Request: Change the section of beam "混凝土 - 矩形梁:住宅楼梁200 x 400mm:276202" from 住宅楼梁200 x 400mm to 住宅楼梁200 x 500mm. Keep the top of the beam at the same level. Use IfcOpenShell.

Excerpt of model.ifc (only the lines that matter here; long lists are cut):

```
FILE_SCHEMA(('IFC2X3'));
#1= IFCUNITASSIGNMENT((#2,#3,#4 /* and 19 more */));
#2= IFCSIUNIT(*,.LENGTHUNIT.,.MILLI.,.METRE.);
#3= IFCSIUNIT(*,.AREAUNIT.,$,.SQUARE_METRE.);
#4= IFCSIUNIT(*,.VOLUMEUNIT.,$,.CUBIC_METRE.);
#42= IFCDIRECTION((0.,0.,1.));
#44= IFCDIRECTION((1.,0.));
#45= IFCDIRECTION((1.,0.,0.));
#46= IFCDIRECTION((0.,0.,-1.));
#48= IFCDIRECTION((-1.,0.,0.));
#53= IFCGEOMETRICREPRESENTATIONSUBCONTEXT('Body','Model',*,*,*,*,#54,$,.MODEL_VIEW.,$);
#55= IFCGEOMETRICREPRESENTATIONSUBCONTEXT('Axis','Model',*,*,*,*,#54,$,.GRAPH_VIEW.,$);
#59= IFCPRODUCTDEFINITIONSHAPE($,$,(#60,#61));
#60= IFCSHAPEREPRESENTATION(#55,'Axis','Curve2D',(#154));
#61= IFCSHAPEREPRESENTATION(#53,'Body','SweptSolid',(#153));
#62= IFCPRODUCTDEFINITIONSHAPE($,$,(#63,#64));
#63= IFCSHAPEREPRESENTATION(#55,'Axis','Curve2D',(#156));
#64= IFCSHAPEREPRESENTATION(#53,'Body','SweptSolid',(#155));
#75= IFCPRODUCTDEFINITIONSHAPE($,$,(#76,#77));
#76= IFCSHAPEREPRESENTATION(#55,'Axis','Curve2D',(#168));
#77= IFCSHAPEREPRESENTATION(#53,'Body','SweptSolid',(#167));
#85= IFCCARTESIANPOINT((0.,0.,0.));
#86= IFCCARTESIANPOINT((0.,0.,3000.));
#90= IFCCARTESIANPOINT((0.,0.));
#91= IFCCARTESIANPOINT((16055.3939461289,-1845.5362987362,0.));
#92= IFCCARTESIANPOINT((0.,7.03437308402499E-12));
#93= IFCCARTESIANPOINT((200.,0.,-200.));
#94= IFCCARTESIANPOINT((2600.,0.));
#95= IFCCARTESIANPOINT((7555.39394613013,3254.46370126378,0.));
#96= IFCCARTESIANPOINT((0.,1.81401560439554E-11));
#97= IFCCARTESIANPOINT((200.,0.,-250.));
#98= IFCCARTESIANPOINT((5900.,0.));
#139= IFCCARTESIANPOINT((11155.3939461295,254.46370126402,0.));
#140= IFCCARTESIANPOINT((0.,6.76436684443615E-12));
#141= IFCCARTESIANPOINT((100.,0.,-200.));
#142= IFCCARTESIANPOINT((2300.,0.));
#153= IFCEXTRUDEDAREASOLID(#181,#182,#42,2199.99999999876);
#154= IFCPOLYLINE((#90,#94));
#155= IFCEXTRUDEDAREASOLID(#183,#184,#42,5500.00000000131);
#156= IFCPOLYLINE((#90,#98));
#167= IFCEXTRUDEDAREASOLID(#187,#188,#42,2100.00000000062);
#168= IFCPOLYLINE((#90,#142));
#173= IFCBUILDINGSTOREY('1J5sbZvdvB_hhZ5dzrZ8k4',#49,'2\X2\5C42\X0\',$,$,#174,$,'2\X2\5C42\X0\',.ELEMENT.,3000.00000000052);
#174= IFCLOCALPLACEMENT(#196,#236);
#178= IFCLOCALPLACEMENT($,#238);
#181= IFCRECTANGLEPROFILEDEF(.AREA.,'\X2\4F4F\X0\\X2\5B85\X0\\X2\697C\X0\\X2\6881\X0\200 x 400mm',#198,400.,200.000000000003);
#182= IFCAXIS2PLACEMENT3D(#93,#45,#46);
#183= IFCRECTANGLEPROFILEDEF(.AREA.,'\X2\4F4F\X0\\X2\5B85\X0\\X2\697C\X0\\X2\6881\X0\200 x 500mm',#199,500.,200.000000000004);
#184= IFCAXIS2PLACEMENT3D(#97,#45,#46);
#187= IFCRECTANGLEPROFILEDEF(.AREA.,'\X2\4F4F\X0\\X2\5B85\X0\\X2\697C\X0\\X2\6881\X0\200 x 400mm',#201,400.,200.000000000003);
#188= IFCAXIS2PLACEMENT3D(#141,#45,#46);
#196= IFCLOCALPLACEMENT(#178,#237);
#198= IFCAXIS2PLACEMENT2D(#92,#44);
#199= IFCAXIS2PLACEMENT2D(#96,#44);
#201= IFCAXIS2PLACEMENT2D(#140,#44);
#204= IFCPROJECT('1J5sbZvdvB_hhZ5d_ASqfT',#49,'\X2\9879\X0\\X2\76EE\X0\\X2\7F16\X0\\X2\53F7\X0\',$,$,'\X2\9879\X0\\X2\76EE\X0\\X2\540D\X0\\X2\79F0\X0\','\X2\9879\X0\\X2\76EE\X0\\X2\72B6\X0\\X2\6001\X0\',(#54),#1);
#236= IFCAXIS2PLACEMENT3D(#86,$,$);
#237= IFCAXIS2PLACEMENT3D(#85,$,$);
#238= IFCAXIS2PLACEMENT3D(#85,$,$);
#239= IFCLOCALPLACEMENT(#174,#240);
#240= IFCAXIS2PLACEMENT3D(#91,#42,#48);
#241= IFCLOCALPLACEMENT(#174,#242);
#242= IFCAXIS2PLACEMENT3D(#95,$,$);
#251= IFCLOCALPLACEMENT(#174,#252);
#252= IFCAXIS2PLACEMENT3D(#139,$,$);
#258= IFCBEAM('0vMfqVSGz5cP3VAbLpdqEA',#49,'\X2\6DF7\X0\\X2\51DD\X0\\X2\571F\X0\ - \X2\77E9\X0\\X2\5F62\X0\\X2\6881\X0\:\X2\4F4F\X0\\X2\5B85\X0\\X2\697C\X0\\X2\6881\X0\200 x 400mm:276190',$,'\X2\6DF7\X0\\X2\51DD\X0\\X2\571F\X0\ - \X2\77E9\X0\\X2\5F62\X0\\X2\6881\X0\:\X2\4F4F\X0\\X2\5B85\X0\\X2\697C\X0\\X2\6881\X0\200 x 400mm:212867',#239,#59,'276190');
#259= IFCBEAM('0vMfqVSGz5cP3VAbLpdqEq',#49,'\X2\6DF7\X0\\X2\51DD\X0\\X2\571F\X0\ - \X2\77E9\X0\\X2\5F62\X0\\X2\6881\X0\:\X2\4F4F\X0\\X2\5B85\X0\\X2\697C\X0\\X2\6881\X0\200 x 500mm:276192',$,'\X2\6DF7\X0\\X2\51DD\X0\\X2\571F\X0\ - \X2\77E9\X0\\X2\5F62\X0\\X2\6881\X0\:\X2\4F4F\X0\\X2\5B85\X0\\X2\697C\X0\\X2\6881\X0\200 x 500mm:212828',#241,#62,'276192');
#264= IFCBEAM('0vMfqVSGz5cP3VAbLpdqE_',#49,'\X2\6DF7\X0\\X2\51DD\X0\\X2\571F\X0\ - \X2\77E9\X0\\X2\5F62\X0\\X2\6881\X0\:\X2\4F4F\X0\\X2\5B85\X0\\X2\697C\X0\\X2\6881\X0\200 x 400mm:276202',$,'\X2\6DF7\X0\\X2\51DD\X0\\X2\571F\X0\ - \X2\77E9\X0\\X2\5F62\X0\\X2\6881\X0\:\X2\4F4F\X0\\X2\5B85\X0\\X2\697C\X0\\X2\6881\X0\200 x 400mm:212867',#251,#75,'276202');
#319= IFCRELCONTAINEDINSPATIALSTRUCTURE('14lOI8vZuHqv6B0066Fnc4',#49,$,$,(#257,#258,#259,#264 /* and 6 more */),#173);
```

```python
import ifcopenshell
import ifcopenshell.util.element
import ifcopenshell.util.representation

model = ifcopenshell.open("model.ifc")

member = model.by_guid("0vMfqVSGz5cP3VAbLpdqE_")
source = next(p for p in model.by_type("IfcRectangleProfileDef") if p.ProfileName == "住宅楼梁200 x 500mm")

body = ifcopenshell.util.representation.get_representation(member, "Model", "Body")
solid = body.Items[0]
old_profile = solid.SweptArea

# Copy the section's sizes but keep this member's own profile position.
profile = ifcopenshell.util.element.copy(model, source)
# Profiles are centred, so shift by half the change in depth to hold the top.
shift = (old_profile.XDim - profile.XDim) / 2
x, y = old_profile.Position.Location.Coordinates
up = (-1.0, 0.0)  # upwards, in the solid's own plane
location = model.createIfcCartesianPoint((x + up[0] * shift, y + up[1] * shift))
profile.Position = model.createIfcAxis2Placement2D(location, old_profile.Position.RefDirection)
solid.SweptArea = profile
if not model.get_total_inverses(old_profile):
    ifcopenshell.util.element.remove_deep2(model, old_profile)
member.Name = member.Name.replace("住宅楼梁200 x 400mm", "住宅楼梁200 x 500mm")
member.ObjectType = member.ObjectType.replace("住宅楼梁200 x 400mm", "住宅楼梁200 x 500mm")

print(solid.SweptArea)

model.write("model_updated.ifc")
```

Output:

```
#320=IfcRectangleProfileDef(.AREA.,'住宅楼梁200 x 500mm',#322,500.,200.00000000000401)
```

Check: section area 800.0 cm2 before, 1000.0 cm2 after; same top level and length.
